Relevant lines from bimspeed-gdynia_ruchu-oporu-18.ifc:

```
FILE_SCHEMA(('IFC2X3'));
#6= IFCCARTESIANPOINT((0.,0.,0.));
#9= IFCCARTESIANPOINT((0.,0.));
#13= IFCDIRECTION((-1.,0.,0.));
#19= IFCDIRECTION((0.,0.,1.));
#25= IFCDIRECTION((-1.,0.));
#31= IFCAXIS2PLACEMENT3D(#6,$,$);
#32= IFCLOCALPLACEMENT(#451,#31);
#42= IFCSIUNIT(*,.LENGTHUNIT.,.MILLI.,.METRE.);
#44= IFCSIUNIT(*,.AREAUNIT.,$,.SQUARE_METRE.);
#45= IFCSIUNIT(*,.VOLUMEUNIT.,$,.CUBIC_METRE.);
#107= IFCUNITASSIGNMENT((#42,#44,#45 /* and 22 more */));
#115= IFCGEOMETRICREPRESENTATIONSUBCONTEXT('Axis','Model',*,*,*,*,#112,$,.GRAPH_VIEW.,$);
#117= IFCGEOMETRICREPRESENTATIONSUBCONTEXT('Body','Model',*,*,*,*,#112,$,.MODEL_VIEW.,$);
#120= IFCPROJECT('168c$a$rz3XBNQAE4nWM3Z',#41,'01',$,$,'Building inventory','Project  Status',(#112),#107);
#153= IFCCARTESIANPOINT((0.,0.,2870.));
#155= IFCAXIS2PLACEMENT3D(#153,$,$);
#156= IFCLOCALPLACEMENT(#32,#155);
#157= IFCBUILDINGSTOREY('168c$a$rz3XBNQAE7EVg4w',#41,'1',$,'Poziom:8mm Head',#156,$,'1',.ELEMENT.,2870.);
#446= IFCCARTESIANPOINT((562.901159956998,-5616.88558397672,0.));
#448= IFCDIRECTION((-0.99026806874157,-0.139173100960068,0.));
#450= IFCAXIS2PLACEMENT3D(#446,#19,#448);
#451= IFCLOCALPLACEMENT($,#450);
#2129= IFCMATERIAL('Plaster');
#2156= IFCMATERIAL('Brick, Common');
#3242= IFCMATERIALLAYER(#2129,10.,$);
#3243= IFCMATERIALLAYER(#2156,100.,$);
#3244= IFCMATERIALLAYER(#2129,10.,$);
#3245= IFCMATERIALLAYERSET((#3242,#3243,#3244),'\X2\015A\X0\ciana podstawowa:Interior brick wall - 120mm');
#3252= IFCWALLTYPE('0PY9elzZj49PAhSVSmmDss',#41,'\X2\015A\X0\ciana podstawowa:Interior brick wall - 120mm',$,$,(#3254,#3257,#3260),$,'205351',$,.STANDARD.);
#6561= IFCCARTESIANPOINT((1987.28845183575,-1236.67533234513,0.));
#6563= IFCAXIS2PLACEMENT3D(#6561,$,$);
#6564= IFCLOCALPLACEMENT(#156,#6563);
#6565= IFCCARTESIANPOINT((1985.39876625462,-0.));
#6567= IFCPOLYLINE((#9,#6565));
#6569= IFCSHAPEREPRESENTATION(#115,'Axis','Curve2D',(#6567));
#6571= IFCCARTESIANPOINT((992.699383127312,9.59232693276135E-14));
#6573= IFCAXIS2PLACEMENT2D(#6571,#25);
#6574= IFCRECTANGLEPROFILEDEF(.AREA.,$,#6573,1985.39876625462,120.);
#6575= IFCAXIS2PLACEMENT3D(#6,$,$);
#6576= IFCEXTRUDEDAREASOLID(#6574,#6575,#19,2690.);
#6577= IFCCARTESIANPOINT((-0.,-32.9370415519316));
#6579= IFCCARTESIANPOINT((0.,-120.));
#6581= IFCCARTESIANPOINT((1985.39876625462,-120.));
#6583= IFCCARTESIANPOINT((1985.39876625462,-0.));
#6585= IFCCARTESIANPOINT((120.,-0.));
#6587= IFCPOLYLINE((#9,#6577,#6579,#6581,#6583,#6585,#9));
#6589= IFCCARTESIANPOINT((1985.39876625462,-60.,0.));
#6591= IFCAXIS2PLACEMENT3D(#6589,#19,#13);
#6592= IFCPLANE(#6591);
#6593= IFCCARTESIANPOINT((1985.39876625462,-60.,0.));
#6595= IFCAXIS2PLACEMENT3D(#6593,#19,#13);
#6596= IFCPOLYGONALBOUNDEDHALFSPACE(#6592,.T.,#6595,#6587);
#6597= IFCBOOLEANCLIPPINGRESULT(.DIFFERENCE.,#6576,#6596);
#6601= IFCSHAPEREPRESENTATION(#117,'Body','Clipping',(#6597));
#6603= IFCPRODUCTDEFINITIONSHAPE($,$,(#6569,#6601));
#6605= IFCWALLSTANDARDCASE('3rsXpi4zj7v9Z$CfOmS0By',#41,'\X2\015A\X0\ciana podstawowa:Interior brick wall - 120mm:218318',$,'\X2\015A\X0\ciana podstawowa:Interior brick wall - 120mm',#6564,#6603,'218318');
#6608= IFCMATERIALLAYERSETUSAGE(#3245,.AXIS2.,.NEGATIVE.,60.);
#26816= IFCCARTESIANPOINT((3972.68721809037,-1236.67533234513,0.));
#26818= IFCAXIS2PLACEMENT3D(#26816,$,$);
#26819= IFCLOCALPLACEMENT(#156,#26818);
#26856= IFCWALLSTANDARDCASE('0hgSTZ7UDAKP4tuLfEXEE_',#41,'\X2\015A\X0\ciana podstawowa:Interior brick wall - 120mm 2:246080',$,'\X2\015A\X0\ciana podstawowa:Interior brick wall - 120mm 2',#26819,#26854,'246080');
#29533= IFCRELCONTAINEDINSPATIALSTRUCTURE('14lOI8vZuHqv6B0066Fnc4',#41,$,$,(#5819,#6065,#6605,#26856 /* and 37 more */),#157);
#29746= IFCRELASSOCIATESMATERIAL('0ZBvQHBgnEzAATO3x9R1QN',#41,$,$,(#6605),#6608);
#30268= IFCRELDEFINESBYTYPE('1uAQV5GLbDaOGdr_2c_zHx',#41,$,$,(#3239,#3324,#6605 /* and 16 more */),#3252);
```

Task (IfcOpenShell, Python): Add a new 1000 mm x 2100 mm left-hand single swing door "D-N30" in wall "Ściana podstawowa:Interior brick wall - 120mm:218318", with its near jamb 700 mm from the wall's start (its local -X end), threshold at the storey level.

```python
import numpy as np
import ifcopenshell
import ifcopenshell.api.feature
import ifcopenshell.api.geometry
import ifcopenshell.api.root
import ifcopenshell.api.spatial
import ifcopenshell.api.type
import ifcopenshell.geom
import ifcopenshell.util.element
import ifcopenshell.util.placement
import ifcopenshell.util.representation
import ifcopenshell.util.shape
import ifcopenshell.util.unit

model = ifcopenshell.open("bimspeed-gdynia_ruchu-oporu-18.ifc")
unit_scale = ifcopenshell.util.unit.calculate_unit_scale(model)
settings = ifcopenshell.geom.settings()


def volume(element):
    """Net volume in cubic metres, openings subtracted."""
    shape = ifcopenshell.geom.create_shape(settings, element)
    return ifcopenshell.util.shape.get_volume(shape.geometry)


wall = model.by_guid("3rsXpi4zj7v9Z$CfOmS0By")
storey = ifcopenshell.util.element.get_container(wall, ifc_class="IfcBuildingStorey")
context = ifcopenshell.util.representation.get_context(model, "Model", "Body", "MODEL_VIEW")
before = volume(wall)

width, height, from_end, sill = 1, 2.1, 0.7, 0.0  # metres

# The wall runs along its own X axis, and the end named is its -X end.
wall_shape = ifcopenshell.geom.create_shape(settings, wall)
x, y, z = ifcopenshell.util.shape.get_vertices(wall_shape.geometry).T
start = x.min() + from_end
face, thickness = float(y.min()), float(y.max() - y.min())
wall_matrix = ifcopenshell.util.placement.get_local_placement(wall.ObjectPlacement)
level = ifcopenshell.util.placement.get_local_placement(storey.ObjectPlacement)[2, 3]


def in_wall(x, y):
    """Placement at x, y metres in the wall's axes, at sill height."""
    matrix = wall_matrix.copy()
    matrix[:, 3] = wall_matrix @ np.array([x / unit_scale, y / unit_scale, 0.0, 1.0])
    matrix[2, 3] = level + sill / unit_scale
    return matrix


# Opening: a box that overshoots both wall faces by 50 mm.
opening = ifcopenshell.api.root.create_entity(model, ifc_class="IfcOpeningElement")
box = ifcopenshell.api.geometry.add_wall_representation(
    model, context=context, length=width, height=height, thickness=thickness + 0.1
)
ifcopenshell.api.geometry.assign_representation(model, product=opening, representation=box)
ifcopenshell.api.geometry.edit_object_placement(model, product=opening, matrix=in_wall(start, face - 0.05), is_si=False)
ifcopenshell.api.feature.add_feature(model, feature=opening, element=wall)

door = ifcopenshell.api.root.create_entity(model, ifc_class="IfcDoor", name="D-N30")
door.OverallWidth, door.OverallHeight = width / unit_scale, height / unit_scale
body = ifcopenshell.api.geometry.add_door_representation(
    model,
    context=context,
    overall_width=door.OverallWidth,
    overall_height=door.OverallHeight,
    operation_type="SINGLE_SWING_LEFT",
    lining_properties={"LiningDepth": thickness / unit_scale, "ThresholdDepth": thickness / unit_scale},
)
ifcopenshell.api.geometry.assign_representation(model, product=door, representation=body)
ifcopenshell.api.spatial.assign_container(model, products=[door], relating_structure=storey)
fills = ifcopenshell.api.feature.add_filling(model, opening=opening, element=door)
fills.OwnerHistory = door.OwnerHistory  # required in IFC2X3

# IFC2X3 keeps the operation on the door style.
style = ifcopenshell.api.root.create_entity(model, ifc_class="IfcDoorStyle", name="D-N30")
style.OperationType, style.ConstructionType = "SINGLE_SWING_LEFT", "NOTDEFINED"
style.ParameterTakesPrecedence = style.Sizeable = False
ifcopenshell.api.type.assign_type(model, related_objects=[door], relating_type=style)

# The lining spans the wall, so the door starts at the wall face.
ifcopenshell.api.geometry.edit_object_placement(model, product=door, matrix=in_wall(start, face), is_si=False)

after = volume(wall)

print(f"wall volume {before:.3f} -> {after:.3f} m3")

model.write("bimspeed-gdynia_ruchu-oporu-18_updated.ifc")
```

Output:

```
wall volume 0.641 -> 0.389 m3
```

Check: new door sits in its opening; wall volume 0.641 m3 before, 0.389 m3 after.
